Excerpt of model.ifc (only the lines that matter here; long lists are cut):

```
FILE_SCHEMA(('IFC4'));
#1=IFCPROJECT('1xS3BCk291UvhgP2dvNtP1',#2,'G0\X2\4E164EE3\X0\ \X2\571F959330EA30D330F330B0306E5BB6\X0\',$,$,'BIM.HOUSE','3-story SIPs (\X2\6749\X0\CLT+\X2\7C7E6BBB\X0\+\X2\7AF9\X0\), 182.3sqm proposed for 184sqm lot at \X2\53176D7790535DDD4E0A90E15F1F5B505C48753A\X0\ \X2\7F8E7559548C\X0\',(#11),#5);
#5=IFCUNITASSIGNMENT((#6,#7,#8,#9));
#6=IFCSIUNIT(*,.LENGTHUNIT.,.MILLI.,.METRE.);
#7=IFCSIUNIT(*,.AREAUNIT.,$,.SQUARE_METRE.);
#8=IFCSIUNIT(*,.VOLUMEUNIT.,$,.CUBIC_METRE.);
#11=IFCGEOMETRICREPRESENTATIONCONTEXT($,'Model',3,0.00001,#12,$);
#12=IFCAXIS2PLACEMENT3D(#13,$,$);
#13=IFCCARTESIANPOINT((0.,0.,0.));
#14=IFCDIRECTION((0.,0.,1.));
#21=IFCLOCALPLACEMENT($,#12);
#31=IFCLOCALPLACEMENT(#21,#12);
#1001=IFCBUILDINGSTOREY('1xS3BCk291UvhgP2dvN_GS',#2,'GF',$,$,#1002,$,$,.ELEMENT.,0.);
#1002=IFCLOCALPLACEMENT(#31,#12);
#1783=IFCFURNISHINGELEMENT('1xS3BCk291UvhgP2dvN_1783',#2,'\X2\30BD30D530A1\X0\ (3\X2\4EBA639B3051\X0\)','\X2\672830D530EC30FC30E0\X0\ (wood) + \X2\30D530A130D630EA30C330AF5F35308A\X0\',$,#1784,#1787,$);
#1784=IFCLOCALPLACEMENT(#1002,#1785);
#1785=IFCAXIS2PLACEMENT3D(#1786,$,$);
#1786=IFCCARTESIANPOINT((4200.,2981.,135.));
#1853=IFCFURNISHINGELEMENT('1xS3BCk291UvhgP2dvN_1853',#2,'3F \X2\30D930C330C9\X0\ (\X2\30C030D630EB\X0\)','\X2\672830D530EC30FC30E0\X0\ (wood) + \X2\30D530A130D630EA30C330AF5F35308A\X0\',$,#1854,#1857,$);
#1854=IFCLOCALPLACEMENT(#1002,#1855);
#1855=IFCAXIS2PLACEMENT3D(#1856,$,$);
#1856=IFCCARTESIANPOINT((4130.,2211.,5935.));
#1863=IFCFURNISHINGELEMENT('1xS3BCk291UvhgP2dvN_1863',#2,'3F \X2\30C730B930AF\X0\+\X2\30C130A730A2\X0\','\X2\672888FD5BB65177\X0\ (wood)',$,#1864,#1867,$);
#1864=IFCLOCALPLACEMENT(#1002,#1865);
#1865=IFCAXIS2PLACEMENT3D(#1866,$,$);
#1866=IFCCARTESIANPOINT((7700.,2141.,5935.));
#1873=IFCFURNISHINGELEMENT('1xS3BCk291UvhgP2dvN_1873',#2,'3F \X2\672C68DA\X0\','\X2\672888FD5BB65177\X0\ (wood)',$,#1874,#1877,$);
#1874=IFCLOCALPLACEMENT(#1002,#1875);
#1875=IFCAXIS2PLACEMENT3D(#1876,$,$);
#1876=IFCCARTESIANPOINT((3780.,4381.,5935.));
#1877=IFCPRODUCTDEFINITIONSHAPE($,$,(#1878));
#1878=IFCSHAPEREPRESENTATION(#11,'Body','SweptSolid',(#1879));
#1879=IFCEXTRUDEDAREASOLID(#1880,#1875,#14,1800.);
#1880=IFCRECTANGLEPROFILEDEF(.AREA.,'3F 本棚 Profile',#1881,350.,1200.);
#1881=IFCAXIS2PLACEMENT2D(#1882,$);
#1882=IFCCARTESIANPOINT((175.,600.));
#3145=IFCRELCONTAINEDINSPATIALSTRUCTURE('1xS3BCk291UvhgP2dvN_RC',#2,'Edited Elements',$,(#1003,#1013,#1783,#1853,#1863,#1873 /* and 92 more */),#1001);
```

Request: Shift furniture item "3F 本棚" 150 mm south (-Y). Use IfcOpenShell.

```python
import ifcopenshell
import ifcopenshell.api.geometry
import ifcopenshell.util.placement
import ifcopenshell.util.unit

model = ifcopenshell.open("model.ifc")
unit_scale = ifcopenshell.util.unit.calculate_unit_scale(model)

item = model.by_id(1873)
matrix = ifcopenshell.util.placement.get_local_placement(item.ObjectPlacement)
matrix[1, 3] -= 0.15 / unit_scale
ifcopenshell.api.geometry.edit_object_placement(model, product=item, matrix=matrix, is_si=False)

print(ifcopenshell.util.placement.get_local_placement(item.ObjectPlacement).round(3) + 0.0)

model.write("model-out.ifc")
```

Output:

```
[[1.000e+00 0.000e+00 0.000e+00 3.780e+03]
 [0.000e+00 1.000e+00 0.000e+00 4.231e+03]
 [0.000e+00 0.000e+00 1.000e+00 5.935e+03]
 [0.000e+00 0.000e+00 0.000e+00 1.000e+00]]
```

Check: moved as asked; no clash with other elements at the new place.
